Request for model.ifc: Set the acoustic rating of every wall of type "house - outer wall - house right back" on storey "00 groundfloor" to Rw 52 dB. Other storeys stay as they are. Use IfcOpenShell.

First a look at what the model holds.

```python
import ifcopenshell
import ifcopenshell.util.element

model = ifcopenshell.open("model.ifc")
print(model.schema)
storey = next(s for s in model.by_type("IfcBuildingStorey") if s.Name == "00 groundfloor")
walls = [e for e in ifcopenshell.util.element.get_decomposition(storey) if e.is_a("IfcWall")]
seen = {}
for e in walls:
    element_type = ifcopenshell.util.element.get_type(e)
    key = (element_type.Name if element_type != e and element_type else None, ifcopenshell.util.element.get_pset(e, "Pset_WallCommon", "AcousticRating"))
    seen[key] = seen.get(key, 0) + 1
for (name, value), count in sorted(seen.items(), key=str):
    print(count, "x", name, "|", value)
```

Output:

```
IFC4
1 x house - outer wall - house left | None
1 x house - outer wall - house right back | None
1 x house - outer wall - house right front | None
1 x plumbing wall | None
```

```python
import ifcopenshell
import ifcopenshell.api.pset
import ifcopenshell.util.element

model = ifcopenshell.open("model.ifc")

storey = next(s for s in model.by_type("IfcBuildingStorey") if s.Name == "00 groundfloor")
walls = [e for e in ifcopenshell.util.element.get_decomposition(storey) if e.is_a("IfcWall")]

count = 0
for e in walls:
    element_type = ifcopenshell.util.element.get_type(e)
    if element_type in (None, e) or element_type.Name != "house - outer wall - house right back":
        continue
    # add_pset returns the element's existing set when there is one.
    pset = ifcopenshell.api.pset.add_pset(model, product=e, name="Pset_WallCommon")
    ifcopenshell.api.pset.edit_pset(model, pset=pset, properties={"AcousticRating": "Rw 52 dB"})
    count += 1

print(count, "walls updated")

model.write("model_updated.ifc")
```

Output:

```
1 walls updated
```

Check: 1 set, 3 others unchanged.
